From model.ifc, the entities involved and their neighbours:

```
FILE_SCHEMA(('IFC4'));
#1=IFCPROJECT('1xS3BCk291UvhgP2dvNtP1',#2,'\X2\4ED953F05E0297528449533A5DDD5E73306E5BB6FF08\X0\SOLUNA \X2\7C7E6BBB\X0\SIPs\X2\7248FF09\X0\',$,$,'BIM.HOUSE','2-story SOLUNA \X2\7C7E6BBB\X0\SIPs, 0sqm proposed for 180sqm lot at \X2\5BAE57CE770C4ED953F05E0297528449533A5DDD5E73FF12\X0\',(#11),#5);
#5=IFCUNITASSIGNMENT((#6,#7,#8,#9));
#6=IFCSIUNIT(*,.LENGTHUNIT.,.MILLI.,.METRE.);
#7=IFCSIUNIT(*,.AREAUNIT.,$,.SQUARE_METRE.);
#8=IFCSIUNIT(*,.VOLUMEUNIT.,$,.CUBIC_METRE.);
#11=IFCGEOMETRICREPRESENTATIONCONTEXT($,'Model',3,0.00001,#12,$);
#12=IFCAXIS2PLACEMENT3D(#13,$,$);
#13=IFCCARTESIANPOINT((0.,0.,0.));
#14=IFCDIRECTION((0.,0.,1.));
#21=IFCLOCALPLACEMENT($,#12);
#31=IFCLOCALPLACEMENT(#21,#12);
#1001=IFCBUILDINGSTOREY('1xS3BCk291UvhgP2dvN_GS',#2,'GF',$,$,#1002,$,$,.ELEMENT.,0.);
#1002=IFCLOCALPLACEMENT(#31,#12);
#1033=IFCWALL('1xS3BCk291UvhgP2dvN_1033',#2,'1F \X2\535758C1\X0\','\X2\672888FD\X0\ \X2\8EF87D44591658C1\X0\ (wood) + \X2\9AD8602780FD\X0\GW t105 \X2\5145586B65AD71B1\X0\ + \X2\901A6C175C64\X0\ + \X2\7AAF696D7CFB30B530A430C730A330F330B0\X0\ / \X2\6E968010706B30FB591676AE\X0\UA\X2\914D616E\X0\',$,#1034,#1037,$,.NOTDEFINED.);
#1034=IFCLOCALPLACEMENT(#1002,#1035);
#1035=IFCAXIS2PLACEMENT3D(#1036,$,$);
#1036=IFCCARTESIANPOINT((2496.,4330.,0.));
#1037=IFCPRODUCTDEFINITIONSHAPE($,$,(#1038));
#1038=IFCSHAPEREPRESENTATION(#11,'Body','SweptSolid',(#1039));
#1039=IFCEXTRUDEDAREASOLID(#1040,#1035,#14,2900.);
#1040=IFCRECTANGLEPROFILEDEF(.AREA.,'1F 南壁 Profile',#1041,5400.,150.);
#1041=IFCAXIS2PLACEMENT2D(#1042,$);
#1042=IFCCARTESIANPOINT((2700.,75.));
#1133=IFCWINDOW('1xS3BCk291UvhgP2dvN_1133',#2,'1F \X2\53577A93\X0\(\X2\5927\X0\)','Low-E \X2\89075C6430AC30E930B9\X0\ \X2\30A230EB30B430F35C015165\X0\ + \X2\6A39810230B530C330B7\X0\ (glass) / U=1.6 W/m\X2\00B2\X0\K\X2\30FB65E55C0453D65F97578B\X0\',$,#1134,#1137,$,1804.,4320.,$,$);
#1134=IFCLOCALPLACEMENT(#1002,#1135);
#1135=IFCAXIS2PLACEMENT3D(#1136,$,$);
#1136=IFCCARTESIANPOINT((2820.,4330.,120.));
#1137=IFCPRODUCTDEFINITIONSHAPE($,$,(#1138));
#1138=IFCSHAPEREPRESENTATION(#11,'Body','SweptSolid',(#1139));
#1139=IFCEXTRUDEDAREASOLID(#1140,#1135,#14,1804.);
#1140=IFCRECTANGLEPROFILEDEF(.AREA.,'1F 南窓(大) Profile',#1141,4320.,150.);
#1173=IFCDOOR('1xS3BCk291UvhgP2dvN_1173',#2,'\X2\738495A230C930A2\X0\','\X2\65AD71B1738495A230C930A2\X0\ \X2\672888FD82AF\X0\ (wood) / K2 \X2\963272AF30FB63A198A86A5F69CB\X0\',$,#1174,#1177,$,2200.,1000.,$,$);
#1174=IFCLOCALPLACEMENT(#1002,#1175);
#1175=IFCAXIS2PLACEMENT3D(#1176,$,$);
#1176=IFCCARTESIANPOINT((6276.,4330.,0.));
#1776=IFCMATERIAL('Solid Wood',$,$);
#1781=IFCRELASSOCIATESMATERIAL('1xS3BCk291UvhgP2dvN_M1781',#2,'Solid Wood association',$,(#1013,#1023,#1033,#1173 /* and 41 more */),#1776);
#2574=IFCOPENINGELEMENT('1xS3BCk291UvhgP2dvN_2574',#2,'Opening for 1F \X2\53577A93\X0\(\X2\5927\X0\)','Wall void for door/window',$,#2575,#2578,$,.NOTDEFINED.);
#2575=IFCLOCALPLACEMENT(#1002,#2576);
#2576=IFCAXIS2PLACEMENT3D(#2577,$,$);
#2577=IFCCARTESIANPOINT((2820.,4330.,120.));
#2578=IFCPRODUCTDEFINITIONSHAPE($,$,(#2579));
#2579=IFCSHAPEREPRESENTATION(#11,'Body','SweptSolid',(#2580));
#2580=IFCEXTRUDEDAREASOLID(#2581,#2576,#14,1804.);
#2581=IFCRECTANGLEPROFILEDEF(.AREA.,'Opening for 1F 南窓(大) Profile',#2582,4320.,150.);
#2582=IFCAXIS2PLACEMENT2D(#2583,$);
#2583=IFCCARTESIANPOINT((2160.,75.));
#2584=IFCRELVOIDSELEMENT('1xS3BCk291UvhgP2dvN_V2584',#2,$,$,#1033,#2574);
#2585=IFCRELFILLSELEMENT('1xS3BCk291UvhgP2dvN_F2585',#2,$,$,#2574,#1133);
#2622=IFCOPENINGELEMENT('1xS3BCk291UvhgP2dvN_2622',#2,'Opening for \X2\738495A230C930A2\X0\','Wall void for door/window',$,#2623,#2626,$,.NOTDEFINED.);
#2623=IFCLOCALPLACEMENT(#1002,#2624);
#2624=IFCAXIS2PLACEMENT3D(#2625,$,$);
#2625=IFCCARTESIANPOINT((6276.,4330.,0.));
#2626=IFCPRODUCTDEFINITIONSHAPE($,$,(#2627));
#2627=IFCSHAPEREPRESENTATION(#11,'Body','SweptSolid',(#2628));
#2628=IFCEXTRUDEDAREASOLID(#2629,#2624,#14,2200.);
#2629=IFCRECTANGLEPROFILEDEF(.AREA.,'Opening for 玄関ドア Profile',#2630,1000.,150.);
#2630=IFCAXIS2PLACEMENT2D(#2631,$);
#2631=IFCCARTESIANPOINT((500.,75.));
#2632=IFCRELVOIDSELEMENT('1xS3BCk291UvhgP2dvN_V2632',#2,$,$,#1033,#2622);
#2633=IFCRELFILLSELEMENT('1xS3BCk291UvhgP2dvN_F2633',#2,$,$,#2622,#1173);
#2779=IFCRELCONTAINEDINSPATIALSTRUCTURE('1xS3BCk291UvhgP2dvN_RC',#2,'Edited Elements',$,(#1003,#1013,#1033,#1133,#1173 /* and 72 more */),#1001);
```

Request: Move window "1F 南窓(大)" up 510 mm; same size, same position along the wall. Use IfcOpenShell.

```python
import numpy as np
import ifcopenshell
import ifcopenshell.api.geometry
import ifcopenshell.util.placement
import ifcopenshell.util.unit

model = ifcopenshell.open("model.ifc")
unit_scale = ifcopenshell.util.unit.calculate_unit_scale(model)

window = model.by_id(1133)
opening = window.FillsVoids[0].RelatingOpeningElement
dz = 0.51 / unit_scale

shift = np.array([0.0, 0.0, dz])
# The window is not placed relative to its opening, so move both.
for product in (opening, window):
    matrix = ifcopenshell.util.placement.get_local_placement(product.ObjectPlacement)
    matrix[:3, 3] += shift
    ifcopenshell.api.geometry.edit_object_placement(model, product=product, matrix=matrix, is_si=False)

print(f"moved by {dz * unit_scale:+.3f} m")

model.write("model_edited.ifc")
```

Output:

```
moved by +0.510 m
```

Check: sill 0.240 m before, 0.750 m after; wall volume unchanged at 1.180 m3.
